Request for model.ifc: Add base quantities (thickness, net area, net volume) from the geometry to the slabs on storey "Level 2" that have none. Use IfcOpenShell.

First a look at what the model holds.

```python
import ifcopenshell
import ifcopenshell.util.element
import ifcopenshell.util.unit

model = ifcopenshell.open("model.ifc")
print(model.schema)
for unit_type in ("LENGTHUNIT", "AREAUNIT", "VOLUMEUNIT"):
    print(unit_type, ifcopenshell.util.unit.calculate_unit_scale(model, unit_type))
storey = next(s for s in model.by_type("IfcBuildingStorey") if s.Name == "Level 2")
slabs = [e for e in ifcopenshell.util.element.get_decomposition(storey) if e.is_a("IfcSlab")]
for e in sorted(slabs, key=lambda e: e.id()):
    print(e.id(), e.is_a(), e.Name, list(ifcopenshell.util.element.get_psets(e, qtos_only=True)), sep=" | ")
```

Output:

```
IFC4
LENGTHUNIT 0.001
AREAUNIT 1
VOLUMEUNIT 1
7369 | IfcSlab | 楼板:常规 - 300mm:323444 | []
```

```python
import ifcopenshell
import ifcopenshell.api.pset
import ifcopenshell.geom
import ifcopenshell.util.element
import ifcopenshell.util.shape
import ifcopenshell.util.unit

model = ifcopenshell.open("model.ifc")
unit_scale = ifcopenshell.util.unit.calculate_unit_scale(model)
area_scale = ifcopenshell.util.unit.calculate_unit_scale(model, "AREAUNIT")
volume_scale = ifcopenshell.util.unit.calculate_unit_scale(model, "VOLUMEUNIT")
settings = ifcopenshell.geom.settings()

storey = next(s for s in model.by_type("IfcBuildingStorey") if s.Name == "Level 2")
slabs = [e for e in ifcopenshell.util.element.get_decomposition(storey) if e.is_a("IfcSlab")]

for e in sorted(slabs, key=lambda e: e.id()):
    if ifcopenshell.util.element.get_psets(e, qtos_only=True, should_inherit=False):
        continue
    # Geometry comes back in metres, in the element's own axes.
    shape = ifcopenshell.geom.create_shape(settings, e)
    values = {
        "Width": ifcopenshell.util.shape.get_z(shape.geometry) / unit_scale,
        "NetArea": ifcopenshell.util.shape.get_footprint_area(shape.geometry) / area_scale,
        "NetVolume": ifcopenshell.util.shape.get_volume(shape.geometry) / volume_scale,
    }
    qto = ifcopenshell.api.pset.add_qto(model, product=e, name="Qto_SlabBaseQuantities")
    ifcopenshell.api.pset.edit_qto(model, qto=qto, properties=values)
    print(e.id(), {k: round(v, 3) for k, v in values.items()})

model.write("model_updated.ifc")
```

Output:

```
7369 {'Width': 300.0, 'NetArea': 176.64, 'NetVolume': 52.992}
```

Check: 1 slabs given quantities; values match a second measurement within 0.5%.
